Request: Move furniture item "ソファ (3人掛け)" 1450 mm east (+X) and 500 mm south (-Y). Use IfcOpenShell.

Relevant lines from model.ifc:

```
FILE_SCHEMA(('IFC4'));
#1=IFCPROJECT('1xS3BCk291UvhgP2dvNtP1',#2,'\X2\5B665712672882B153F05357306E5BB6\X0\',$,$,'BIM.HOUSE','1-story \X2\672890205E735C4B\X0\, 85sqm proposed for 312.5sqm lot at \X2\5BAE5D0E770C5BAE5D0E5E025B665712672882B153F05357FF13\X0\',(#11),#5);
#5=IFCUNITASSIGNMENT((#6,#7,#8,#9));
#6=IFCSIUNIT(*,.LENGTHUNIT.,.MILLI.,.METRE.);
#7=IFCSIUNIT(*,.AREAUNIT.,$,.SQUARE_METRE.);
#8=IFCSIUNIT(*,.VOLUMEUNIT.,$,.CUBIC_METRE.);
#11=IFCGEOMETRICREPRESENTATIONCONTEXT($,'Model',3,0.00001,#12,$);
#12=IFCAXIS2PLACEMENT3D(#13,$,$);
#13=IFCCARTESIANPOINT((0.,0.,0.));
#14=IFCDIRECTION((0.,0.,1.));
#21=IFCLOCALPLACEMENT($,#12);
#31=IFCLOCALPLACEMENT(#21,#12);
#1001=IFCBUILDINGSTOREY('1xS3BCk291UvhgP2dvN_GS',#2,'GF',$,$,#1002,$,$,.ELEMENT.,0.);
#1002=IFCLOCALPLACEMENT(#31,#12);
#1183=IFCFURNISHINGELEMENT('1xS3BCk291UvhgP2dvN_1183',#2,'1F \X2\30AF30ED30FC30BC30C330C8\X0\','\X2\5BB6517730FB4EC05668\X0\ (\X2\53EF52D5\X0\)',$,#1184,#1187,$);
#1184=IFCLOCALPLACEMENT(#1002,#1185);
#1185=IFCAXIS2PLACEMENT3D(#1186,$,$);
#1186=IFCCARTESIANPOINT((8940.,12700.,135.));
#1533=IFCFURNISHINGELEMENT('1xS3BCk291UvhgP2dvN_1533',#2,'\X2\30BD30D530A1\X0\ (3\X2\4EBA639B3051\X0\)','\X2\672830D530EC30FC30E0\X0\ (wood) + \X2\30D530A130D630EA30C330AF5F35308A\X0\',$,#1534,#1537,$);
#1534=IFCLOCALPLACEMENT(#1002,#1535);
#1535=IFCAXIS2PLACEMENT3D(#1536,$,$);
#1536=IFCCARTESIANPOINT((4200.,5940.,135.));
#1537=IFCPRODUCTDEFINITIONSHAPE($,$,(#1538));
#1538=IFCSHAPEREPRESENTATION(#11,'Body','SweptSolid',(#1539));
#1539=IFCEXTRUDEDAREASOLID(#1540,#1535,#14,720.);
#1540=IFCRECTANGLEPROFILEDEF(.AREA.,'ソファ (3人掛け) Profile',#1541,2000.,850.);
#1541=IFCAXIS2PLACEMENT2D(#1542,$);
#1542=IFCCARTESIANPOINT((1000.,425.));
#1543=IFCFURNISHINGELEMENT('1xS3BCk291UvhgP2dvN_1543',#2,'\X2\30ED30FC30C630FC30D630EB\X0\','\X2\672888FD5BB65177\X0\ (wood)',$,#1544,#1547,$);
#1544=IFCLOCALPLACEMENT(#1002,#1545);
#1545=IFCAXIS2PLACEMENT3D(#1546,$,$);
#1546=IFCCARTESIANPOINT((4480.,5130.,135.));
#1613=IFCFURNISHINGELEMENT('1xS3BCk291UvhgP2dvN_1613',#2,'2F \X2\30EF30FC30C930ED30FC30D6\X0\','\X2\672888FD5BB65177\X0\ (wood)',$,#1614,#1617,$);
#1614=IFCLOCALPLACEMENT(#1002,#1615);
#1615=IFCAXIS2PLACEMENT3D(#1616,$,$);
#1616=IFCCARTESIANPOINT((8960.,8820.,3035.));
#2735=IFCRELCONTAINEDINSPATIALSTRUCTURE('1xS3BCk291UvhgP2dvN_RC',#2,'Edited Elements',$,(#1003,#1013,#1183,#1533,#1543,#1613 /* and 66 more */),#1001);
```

```python
import ifcopenshell
import ifcopenshell.api.geometry
import ifcopenshell.util.placement
import ifcopenshell.util.unit

model = ifcopenshell.open("model.ifc")
unit_scale = ifcopenshell.util.unit.calculate_unit_scale(model)

item = model.by_guid("1xS3BCk291UvhgP2dvN_1533")
matrix = ifcopenshell.util.placement.get_local_placement(item.ObjectPlacement)
matrix[0, 3] += 1.45 / unit_scale
matrix[1, 3] -= 0.5 / unit_scale
ifcopenshell.api.geometry.edit_object_placement(model, product=item, matrix=matrix, is_si=False)

print(ifcopenshell.util.placement.get_local_placement(item.ObjectPlacement).round(3) + 0.0)

model.write("model_updated.ifc")
```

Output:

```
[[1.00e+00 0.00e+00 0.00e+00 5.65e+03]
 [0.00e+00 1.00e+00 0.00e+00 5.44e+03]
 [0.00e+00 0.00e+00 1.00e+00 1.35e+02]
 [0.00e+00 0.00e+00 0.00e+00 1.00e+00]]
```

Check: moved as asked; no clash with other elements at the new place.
